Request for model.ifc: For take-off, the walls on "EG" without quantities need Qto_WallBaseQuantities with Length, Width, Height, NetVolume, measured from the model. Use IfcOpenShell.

First a look at what the model holds.

```python
import ifcopenshell
import ifcopenshell.util.element
import ifcopenshell.util.unit

model = ifcopenshell.open("model.ifc")
print(model.schema)
for unit_type in ("LENGTHUNIT", "AREAUNIT", "VOLUMEUNIT"):
    print(unit_type, ifcopenshell.util.unit.calculate_unit_scale(model, unit_type))
storey = next(s for s in model.by_type("IfcBuildingStorey") if s.Name == "EG")
walls = [e for e in ifcopenshell.util.element.get_decomposition(storey) if e.is_a("IfcWall")]
for e in sorted(walls, key=lambda e: e.id()):
    print(e.id(), e.is_a(), e.Name, list(ifcopenshell.util.element.get_psets(e, qtos_only=True)), sep=" | ")
```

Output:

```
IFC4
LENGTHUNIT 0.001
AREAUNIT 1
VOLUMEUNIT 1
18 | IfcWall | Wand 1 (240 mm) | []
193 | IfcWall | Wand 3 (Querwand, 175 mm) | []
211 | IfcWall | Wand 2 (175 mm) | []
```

```python
import ifcopenshell
import ifcopenshell.api.pset
import ifcopenshell.geom
import ifcopenshell.util.element
import ifcopenshell.util.shape
import ifcopenshell.util.unit

model = ifcopenshell.open("model.ifc")
unit_scale = ifcopenshell.util.unit.calculate_unit_scale(model)
volume_scale = ifcopenshell.util.unit.calculate_unit_scale(model, "VOLUMEUNIT")
settings = ifcopenshell.geom.settings()

storey = next(s for s in model.by_type("IfcBuildingStorey") if s.Name == "EG")
walls = [e for e in ifcopenshell.util.element.get_decomposition(storey) if e.is_a("IfcWall")]

for e in sorted(walls, key=lambda e: e.id()):
    if ifcopenshell.util.element.get_psets(e, qtos_only=True, should_inherit=False):
        continue
    # Geometry comes back in metres, in the element's own axes.
    shape = ifcopenshell.geom.create_shape(settings, e)
    values = {
        "Length": ifcopenshell.util.shape.get_x(shape.geometry) / unit_scale,
        "Width": ifcopenshell.util.shape.get_y(shape.geometry) / unit_scale,
        "Height": ifcopenshell.util.shape.get_z(shape.geometry) / unit_scale,
        "NetVolume": ifcopenshell.util.shape.get_volume(shape.geometry) / volume_scale,
    }
    qto = ifcopenshell.api.pset.add_qto(model, product=e, name="Qto_WallBaseQuantities")
    ifcopenshell.api.pset.edit_qto(model, qto=qto, properties=values)
    print(e.id(), {k: round(v, 3) for k, v in values.items()})

model.write("model_v2.ifc")
```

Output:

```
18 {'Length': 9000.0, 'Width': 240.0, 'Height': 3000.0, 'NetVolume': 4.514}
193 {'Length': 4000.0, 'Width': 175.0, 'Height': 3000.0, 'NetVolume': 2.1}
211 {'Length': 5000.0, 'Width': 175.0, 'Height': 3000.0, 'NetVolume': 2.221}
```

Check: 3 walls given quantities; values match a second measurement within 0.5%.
